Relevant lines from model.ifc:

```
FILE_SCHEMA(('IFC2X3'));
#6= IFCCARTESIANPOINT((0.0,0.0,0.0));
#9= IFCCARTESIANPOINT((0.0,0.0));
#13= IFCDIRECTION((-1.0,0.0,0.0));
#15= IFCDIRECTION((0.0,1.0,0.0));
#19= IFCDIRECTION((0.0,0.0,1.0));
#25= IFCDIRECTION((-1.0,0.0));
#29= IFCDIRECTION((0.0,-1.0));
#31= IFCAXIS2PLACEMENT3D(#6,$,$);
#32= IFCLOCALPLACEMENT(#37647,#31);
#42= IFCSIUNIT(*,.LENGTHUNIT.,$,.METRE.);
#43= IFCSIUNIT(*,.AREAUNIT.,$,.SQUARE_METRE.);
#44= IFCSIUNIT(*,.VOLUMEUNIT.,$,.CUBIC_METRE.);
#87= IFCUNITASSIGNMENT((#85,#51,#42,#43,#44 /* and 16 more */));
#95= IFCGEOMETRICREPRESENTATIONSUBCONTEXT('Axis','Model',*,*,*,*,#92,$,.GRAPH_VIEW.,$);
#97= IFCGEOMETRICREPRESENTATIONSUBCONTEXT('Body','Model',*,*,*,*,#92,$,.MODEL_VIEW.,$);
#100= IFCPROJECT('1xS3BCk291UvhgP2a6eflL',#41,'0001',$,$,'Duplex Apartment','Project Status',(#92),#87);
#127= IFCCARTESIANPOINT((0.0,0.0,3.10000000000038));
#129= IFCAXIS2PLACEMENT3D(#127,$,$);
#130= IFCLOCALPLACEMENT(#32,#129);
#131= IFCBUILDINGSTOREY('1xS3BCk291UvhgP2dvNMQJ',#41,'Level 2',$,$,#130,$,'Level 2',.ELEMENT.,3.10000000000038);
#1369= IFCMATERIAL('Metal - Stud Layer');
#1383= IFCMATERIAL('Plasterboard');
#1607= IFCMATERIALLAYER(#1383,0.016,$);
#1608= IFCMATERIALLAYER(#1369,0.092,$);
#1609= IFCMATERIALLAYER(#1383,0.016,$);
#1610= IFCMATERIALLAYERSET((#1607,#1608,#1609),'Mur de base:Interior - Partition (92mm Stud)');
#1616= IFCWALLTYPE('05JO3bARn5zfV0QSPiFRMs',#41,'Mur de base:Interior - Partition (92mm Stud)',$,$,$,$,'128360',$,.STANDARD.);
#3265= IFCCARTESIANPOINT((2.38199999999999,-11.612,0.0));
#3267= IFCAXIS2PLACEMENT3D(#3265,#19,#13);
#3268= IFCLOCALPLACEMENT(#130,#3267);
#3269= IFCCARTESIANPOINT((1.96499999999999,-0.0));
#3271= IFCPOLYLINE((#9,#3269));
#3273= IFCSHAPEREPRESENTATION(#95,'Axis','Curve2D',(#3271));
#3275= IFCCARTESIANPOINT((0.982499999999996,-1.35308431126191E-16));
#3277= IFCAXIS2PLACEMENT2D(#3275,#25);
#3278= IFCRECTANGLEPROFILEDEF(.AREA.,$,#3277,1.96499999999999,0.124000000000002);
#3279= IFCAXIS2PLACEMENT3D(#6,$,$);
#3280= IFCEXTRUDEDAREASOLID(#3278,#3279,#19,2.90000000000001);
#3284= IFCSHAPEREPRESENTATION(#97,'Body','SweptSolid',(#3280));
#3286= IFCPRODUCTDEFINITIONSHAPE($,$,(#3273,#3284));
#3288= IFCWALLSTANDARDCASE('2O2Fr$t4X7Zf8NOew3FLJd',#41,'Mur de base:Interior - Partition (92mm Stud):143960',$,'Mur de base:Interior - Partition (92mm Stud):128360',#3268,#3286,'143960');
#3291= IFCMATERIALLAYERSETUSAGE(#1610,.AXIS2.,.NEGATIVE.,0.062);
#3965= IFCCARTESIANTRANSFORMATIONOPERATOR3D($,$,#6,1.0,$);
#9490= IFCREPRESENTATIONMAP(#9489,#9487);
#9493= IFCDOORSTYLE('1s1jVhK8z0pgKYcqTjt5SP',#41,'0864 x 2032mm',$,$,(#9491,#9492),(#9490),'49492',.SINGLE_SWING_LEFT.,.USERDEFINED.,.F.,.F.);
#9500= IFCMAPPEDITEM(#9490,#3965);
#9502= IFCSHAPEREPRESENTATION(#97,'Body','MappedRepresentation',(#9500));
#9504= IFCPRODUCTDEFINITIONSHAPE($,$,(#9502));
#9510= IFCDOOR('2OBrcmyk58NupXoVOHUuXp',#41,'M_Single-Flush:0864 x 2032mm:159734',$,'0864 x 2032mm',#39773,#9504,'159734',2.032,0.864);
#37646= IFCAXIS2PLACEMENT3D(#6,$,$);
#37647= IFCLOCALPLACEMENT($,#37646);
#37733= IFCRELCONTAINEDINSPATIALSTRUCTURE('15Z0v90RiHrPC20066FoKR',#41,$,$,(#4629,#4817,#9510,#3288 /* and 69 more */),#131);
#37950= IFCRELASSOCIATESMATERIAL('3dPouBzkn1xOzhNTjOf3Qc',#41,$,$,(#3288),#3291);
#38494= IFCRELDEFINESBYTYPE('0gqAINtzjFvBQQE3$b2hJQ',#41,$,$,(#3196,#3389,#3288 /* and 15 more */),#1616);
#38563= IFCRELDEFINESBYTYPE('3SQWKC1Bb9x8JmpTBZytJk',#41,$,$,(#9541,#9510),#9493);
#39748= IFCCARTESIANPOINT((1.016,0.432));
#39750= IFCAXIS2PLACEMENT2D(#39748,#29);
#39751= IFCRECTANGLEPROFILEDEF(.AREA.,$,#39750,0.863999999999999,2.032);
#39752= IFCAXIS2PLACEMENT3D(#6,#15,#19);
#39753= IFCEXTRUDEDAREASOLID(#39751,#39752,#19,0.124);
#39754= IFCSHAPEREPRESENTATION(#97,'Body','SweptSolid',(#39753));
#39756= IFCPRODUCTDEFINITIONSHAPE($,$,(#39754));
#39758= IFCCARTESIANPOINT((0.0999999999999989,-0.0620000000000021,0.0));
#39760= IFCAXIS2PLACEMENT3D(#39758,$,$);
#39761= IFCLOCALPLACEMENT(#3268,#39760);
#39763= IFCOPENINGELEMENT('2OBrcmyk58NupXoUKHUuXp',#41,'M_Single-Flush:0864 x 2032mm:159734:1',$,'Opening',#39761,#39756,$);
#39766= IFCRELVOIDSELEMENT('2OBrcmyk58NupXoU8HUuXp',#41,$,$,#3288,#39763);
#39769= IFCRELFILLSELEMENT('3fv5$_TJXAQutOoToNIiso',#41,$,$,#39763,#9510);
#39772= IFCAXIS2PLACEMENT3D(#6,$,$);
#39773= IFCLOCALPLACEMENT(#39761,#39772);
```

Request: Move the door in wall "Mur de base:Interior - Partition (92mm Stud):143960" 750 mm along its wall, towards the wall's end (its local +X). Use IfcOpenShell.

```python
import ifcopenshell
import ifcopenshell.api.geometry
import ifcopenshell.util.placement
import ifcopenshell.util.unit

model = ifcopenshell.open("model.ifc")
unit_scale = ifcopenshell.util.unit.calculate_unit_scale(model)

door = model.by_guid("2OBrcmyk58NupXoVOHUuXp")
opening = door.FillsVoids[0].RelatingOpeningElement
wall = opening.VoidsElements[0].RelatingBuildingElement

wall_matrix = ifcopenshell.util.placement.get_local_placement(wall.ObjectPlacement)
shift = wall_matrix[:3, 0] * 0.75 / unit_scale
before = ifcopenshell.util.placement.get_local_placement(door.ObjectPlacement)[:3, 3].copy()

# The door is placed relative to its opening, so it follows when the opening moves.
matrix = ifcopenshell.util.placement.get_local_placement(opening.ObjectPlacement)
matrix[:3, 3] += shift
ifcopenshell.api.geometry.edit_object_placement(
    model, product=opening, matrix=matrix, is_si=False, should_transform_children=True
)

after = ifcopenshell.util.placement.get_local_placement(door.ObjectPlacement)[:3, 3]
print("door moved by", (after - before).round(3) + 0.0)

model.write("model_rev.ifc")
```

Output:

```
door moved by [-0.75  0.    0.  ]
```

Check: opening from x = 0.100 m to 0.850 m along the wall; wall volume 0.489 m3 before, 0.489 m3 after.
